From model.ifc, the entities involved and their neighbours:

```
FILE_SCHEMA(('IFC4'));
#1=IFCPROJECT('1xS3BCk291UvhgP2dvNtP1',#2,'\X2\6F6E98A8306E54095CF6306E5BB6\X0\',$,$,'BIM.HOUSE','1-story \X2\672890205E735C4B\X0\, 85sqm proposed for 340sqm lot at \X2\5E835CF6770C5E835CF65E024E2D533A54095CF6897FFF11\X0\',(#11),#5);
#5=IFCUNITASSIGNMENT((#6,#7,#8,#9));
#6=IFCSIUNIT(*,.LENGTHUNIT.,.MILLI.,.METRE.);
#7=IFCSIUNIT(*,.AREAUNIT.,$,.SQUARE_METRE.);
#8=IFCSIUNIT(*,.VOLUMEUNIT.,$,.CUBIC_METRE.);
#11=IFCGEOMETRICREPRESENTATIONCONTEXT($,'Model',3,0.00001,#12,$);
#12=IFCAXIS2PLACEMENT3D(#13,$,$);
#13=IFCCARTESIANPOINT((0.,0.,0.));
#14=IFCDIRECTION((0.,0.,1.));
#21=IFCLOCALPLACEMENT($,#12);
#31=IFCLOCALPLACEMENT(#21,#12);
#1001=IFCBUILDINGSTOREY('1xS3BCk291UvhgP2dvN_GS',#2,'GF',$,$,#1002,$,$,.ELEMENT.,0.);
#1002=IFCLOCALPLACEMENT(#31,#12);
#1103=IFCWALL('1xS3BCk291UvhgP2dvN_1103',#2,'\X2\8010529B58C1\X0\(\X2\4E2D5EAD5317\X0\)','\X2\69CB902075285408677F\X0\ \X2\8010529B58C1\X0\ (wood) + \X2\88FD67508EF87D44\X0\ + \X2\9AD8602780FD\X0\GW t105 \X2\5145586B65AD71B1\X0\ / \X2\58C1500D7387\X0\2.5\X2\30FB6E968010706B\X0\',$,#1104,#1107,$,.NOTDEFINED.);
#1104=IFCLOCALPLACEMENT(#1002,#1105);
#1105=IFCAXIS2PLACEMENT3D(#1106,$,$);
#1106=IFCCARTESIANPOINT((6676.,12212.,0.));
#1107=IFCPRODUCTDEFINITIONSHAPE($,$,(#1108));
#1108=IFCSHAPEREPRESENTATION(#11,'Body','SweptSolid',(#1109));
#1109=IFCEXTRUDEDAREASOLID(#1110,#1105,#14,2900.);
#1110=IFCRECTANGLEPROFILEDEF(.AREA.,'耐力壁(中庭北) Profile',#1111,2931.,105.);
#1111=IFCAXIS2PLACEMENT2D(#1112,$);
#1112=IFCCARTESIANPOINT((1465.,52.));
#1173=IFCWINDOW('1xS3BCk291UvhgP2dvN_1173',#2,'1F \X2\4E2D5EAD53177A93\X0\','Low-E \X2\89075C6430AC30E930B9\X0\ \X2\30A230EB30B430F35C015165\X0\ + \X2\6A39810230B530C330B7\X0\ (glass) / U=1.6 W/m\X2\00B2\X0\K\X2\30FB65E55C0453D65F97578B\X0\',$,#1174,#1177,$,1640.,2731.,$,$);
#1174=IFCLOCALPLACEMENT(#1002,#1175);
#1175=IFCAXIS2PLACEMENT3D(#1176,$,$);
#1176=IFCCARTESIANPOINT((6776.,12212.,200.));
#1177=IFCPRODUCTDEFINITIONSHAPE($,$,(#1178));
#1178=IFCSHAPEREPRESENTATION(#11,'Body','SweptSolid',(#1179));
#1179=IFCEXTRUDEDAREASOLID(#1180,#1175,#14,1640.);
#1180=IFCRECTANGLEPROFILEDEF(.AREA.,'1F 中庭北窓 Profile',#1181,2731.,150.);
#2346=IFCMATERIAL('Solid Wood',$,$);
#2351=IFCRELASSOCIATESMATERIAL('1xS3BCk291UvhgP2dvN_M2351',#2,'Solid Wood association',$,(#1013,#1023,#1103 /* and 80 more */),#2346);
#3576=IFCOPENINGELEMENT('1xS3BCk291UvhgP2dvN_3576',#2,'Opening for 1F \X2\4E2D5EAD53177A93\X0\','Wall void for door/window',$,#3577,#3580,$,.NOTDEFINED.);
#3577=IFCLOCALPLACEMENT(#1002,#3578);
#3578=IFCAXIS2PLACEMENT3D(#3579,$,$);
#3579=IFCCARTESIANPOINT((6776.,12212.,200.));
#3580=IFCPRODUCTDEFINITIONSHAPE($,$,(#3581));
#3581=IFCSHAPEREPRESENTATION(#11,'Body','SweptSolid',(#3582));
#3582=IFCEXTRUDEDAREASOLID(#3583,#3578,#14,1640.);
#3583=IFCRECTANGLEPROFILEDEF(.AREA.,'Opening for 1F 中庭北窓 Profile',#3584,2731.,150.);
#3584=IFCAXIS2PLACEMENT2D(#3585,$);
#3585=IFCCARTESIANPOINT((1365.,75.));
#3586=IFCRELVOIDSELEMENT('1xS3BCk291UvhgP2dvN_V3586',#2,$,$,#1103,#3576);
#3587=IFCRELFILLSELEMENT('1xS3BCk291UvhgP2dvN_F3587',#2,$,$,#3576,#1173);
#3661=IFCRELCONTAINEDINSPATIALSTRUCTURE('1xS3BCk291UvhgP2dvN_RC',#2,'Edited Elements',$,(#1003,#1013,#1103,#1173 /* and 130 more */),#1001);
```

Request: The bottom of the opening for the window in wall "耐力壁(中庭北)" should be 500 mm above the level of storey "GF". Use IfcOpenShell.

```python
import numpy as np
import ifcopenshell
import ifcopenshell.api.geometry
import ifcopenshell.geom
import ifcopenshell.util.element
import ifcopenshell.util.placement
import ifcopenshell.util.shape
import ifcopenshell.util.unit

model = ifcopenshell.open("model.ifc")
unit_scale = ifcopenshell.util.unit.calculate_unit_scale(model)

window = model.by_guid("1xS3BCk291UvhgP2dvN_1173")
opening = window.FillsVoids[0].RelatingOpeningElement
storey = ifcopenshell.util.element.get_container(window, ifc_class="IfcBuildingStorey")
level = ifcopenshell.util.placement.get_local_placement(storey.ObjectPlacement)[2, 3]

# The opening's origin need not be at the sill, so measure its lowest point.
shape = ifcopenshell.geom.create_shape(ifcopenshell.geom.settings(), opening)
bottom = ifcopenshell.util.shape.get_shape_bottom_elevation(shape, shape.geometry) / unit_scale
dz = level + 500.0 - bottom

shift = np.array([0.0, 0.0, dz])
# The window is not placed relative to its opening, so move both.
for product in (opening, window):
    matrix = ifcopenshell.util.placement.get_local_placement(product.ObjectPlacement)
    matrix[:3, 3] += shift
    ifcopenshell.api.geometry.edit_object_placement(model, product=product, matrix=matrix, is_si=False)

print(f"moved by {dz * unit_scale:+.3f} m")

model.write("model_rev.ifc")
```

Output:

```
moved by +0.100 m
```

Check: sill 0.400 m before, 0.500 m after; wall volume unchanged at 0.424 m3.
